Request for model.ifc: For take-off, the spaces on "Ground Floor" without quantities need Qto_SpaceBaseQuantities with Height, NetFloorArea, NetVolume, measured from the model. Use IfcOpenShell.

First a look at what the model holds.

```python
import ifcopenshell
import ifcopenshell.util.element
import ifcopenshell.util.unit

model = ifcopenshell.open("model.ifc")
print(model.schema)
for unit_type in ("LENGTHUNIT", "AREAUNIT", "VOLUMEUNIT"):
    print(unit_type, ifcopenshell.util.unit.calculate_unit_scale(model, unit_type))
storey = next(s for s in model.by_type("IfcBuildingStorey") if s.Name == "Ground Floor")
spaces = [e for e in ifcopenshell.util.element.get_decomposition(storey) if e.is_a("IfcSpace")]
for e in sorted(spaces, key=lambda e: e.id()):
    print(e.id(), e.is_a(), e.Name, list(ifcopenshell.util.element.get_psets(e, qtos_only=True)), sep=" | ")
```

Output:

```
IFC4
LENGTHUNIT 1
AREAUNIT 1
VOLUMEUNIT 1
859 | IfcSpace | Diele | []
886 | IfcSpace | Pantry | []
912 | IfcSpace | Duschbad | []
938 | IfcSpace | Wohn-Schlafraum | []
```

```python
import ifcopenshell
import ifcopenshell.api.pset
import ifcopenshell.geom
import ifcopenshell.util.element
import ifcopenshell.util.shape
import ifcopenshell.util.unit

model = ifcopenshell.open("model.ifc")
unit_scale = ifcopenshell.util.unit.calculate_unit_scale(model)
area_scale = ifcopenshell.util.unit.calculate_unit_scale(model, "AREAUNIT")
volume_scale = ifcopenshell.util.unit.calculate_unit_scale(model, "VOLUMEUNIT")
settings = ifcopenshell.geom.settings()

storey = next(s for s in model.by_type("IfcBuildingStorey") if s.Name == "Ground Floor")
spaces = [e for e in ifcopenshell.util.element.get_decomposition(storey) if e.is_a("IfcSpace")]

for e in sorted(spaces, key=lambda e: e.id()):
    if ifcopenshell.util.element.get_psets(e, qtos_only=True, should_inherit=False):
        continue
    # Geometry comes back in metres, in the element's own axes.
    shape = ifcopenshell.geom.create_shape(settings, e)
    values = {
        "Height": ifcopenshell.util.shape.get_z(shape.geometry) / unit_scale,
        "NetFloorArea": ifcopenshell.util.shape.get_footprint_area(shape.geometry) / area_scale,
        "NetVolume": ifcopenshell.util.shape.get_volume(shape.geometry) / volume_scale,
    }
    qto = ifcopenshell.api.pset.add_qto(model, product=e, name="Qto_SpaceBaseQuantities")
    ifcopenshell.api.pset.edit_qto(model, qto=qto, properties=values)
    print(e.id(), {k: round(v, 3) for k, v in values.items()})

model.write("model_rev.ifc")
```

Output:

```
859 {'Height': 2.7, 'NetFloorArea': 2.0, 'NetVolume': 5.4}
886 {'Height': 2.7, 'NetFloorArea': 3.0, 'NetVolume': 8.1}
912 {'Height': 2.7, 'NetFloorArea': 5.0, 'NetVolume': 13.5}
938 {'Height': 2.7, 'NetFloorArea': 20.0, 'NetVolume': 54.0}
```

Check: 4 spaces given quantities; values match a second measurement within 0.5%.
